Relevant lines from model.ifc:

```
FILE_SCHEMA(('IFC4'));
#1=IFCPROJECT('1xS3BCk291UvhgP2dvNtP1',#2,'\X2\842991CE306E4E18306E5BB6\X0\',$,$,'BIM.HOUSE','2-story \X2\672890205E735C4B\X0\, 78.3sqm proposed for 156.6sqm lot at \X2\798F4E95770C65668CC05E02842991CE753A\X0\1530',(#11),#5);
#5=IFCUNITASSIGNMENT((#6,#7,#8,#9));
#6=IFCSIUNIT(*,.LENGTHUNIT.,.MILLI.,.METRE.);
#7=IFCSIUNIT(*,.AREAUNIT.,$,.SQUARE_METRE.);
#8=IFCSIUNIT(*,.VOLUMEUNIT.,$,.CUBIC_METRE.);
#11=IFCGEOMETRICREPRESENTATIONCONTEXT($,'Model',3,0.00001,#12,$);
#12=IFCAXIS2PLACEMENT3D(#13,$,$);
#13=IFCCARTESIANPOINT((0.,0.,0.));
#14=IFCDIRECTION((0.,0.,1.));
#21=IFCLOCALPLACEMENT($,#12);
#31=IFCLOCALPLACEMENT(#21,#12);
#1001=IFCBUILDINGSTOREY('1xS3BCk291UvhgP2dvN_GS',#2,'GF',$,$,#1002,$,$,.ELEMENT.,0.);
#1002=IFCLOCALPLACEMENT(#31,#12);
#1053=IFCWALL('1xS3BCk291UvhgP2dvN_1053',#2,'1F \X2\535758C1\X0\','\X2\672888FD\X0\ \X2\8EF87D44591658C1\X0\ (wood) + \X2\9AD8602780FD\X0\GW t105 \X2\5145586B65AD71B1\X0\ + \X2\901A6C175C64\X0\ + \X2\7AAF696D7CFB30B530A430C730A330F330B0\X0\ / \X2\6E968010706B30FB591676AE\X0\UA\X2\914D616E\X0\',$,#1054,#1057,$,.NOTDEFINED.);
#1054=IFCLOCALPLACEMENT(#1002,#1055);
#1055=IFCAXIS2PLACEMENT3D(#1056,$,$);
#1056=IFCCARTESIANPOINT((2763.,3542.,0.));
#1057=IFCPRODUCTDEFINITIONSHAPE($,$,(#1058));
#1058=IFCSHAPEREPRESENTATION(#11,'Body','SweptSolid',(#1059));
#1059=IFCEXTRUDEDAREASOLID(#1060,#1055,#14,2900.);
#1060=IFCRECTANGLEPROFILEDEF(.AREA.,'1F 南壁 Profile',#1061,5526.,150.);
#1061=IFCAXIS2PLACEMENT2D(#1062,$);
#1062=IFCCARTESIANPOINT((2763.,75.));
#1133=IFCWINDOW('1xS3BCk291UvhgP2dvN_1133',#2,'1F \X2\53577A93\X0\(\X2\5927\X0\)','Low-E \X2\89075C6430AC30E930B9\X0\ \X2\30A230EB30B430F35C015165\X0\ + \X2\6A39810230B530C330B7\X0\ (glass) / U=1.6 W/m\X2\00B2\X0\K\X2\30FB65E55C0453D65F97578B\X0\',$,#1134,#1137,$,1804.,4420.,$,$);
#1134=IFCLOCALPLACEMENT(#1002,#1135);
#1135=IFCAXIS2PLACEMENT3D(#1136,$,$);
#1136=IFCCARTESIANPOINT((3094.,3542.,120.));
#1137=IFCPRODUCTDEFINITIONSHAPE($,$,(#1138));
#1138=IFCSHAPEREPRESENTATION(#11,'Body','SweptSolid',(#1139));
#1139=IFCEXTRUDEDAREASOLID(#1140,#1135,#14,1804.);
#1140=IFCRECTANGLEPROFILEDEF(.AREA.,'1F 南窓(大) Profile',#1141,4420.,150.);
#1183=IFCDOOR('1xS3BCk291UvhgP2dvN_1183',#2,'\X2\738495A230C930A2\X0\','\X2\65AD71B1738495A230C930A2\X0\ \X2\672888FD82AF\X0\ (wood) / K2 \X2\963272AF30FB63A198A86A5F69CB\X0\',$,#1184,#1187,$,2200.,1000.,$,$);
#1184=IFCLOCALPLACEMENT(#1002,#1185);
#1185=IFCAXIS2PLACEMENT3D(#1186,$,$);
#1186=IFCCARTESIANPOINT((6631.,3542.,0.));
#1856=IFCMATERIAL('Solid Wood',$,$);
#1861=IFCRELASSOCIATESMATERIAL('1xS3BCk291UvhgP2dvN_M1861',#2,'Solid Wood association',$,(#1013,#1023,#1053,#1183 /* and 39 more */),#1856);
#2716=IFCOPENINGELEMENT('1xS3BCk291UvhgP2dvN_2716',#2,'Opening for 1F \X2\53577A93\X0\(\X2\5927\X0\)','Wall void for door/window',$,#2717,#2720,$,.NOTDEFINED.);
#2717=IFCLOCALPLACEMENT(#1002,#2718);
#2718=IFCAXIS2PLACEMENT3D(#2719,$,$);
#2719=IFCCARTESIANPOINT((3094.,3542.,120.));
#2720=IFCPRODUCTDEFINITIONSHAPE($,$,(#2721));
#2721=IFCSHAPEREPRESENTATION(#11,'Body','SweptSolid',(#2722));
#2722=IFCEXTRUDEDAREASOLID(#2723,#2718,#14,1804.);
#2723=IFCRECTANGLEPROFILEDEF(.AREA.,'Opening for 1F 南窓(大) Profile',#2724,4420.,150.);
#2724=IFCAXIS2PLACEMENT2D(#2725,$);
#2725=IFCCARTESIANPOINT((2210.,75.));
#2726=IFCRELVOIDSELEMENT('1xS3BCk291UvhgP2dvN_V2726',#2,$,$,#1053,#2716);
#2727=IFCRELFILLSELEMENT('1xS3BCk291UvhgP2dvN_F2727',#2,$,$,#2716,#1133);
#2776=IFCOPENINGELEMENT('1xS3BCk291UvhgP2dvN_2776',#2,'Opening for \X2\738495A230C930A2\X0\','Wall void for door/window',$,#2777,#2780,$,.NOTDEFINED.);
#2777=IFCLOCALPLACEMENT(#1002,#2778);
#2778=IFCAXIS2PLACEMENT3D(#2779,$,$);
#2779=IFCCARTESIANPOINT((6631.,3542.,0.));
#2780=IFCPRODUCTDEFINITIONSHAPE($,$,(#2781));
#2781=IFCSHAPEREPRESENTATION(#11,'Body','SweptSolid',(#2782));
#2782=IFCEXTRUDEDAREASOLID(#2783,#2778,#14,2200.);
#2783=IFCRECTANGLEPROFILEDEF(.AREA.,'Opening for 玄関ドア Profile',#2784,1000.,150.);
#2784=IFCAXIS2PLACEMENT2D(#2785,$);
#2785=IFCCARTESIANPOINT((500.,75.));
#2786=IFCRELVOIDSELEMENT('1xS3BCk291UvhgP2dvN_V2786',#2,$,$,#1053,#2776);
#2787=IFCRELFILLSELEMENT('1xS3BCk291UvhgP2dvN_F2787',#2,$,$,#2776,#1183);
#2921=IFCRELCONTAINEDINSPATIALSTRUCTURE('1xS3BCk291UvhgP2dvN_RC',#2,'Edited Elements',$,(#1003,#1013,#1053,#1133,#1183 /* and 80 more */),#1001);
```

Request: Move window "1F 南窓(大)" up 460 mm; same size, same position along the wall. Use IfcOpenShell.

```python
import numpy as np
import ifcopenshell
import ifcopenshell.api.geometry
import ifcopenshell.util.placement
import ifcopenshell.util.unit

model = ifcopenshell.open("model.ifc")
unit_scale = ifcopenshell.util.unit.calculate_unit_scale(model)

window = model.by_id(1133)
opening = window.FillsVoids[0].RelatingOpeningElement
dz = 460.0

shift = np.array([0.0, 0.0, dz])
# The window is not placed relative to its opening, so move both.
for product in (opening, window):
    matrix = ifcopenshell.util.placement.get_local_placement(product.ObjectPlacement)
    matrix[:3, 3] += shift
    ifcopenshell.api.geometry.edit_object_placement(model, product=product, matrix=matrix, is_si=False)

print(f"moved by {dz * unit_scale:+.3f} m")

model.write("model_updated.ifc")
```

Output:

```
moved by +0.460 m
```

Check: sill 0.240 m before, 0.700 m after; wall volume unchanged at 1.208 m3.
